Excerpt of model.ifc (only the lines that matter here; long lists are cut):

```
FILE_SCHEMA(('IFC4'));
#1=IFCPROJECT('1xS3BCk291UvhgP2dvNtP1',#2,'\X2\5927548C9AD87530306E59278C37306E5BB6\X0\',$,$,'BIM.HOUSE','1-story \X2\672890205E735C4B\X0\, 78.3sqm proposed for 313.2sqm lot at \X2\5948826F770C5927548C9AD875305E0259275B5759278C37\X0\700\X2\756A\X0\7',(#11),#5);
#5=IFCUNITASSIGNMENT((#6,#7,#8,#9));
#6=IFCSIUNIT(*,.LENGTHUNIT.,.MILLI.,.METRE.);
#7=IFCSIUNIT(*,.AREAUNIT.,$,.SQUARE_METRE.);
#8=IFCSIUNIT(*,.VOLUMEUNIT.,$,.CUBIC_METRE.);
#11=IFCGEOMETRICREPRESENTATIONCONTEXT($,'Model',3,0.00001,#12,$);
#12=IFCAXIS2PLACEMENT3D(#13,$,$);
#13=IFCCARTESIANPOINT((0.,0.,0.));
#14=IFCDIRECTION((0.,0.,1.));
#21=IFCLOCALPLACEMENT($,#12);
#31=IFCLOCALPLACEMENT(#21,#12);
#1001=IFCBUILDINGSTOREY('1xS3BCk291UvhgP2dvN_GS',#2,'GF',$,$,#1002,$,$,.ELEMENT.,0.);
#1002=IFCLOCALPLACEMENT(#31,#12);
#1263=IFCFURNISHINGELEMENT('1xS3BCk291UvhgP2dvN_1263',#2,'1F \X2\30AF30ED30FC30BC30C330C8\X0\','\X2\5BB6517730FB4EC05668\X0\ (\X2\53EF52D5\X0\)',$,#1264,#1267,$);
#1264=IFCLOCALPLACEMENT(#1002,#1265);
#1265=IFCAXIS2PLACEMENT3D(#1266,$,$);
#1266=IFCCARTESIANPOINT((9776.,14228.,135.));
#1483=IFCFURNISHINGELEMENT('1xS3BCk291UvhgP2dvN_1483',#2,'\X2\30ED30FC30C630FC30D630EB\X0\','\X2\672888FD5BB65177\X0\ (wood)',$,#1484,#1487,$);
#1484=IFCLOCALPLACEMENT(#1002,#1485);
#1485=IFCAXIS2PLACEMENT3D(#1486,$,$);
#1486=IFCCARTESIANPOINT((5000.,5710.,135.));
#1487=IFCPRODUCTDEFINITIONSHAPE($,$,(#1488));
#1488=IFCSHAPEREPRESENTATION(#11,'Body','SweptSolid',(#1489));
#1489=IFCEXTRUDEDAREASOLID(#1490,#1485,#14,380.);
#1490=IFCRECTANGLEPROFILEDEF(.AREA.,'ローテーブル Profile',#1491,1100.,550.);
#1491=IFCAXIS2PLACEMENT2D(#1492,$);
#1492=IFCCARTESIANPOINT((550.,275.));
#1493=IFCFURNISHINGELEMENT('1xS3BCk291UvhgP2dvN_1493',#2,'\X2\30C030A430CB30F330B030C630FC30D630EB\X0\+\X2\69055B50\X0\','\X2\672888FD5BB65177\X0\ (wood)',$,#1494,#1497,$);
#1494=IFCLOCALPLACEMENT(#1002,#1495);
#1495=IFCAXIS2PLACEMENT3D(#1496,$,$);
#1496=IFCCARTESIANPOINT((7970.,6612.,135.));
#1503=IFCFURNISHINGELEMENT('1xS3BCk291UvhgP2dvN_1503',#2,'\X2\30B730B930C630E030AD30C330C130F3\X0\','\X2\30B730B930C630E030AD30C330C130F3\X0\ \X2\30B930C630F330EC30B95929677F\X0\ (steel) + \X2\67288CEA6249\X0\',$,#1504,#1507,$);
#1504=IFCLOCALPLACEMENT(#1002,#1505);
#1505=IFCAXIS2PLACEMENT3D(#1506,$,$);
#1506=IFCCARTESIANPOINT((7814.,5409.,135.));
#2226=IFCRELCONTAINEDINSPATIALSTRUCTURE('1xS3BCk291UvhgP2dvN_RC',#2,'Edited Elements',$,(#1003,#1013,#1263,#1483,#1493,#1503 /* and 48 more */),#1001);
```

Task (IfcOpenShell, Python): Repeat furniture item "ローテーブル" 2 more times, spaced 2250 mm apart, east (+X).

```python
import numpy as np
import ifcopenshell
import ifcopenshell.api.geometry
import ifcopenshell.api.root
import ifcopenshell.util.element
import ifcopenshell.util.placement
import ifcopenshell.util.unit

model = ifcopenshell.open("model.ifc")
unit_scale = ifcopenshell.util.unit.calculate_unit_scale(model)


def reuse_history(source, copy):
    """copy_class also copies each property set's owner history, people and application; keep the originals."""
    for rel in copy.IsDefinedBy:
        if rel.is_a("IfcRelDefinesByProperties") and (history := rel.RelatingPropertyDefinition.OwnerHistory):
            rel.RelatingPropertyDefinition.OwnerHistory = source.OwnerHistory
            ifcopenshell.util.element.remove_deep2(model, history)


source = model.by_guid("1xS3BCk291UvhgP2dvN_1483")
base = ifcopenshell.util.placement.get_local_placement(source.ObjectPlacement)
step = np.array([1.0, 0.0, 0.0]) * 2.25 / unit_scale

for i in range(1, 3):
    copy = ifcopenshell.api.root.copy_class(model, product=source)
    copy.Representation = ifcopenshell.util.element.copy_deep(
        model, source.Representation, exclude=["IfcGeometricRepresentationContext", "IfcRepresentationMap"]
    )
    reuse_history(source, copy)
    matrix = base.copy()
    matrix[:3, 3] += i * step
    print("added at", matrix[:3, 3].round(3) + 0.0)
    ifcopenshell.api.geometry.edit_object_placement(model, product=copy, matrix=matrix, is_si=False)

model.write("model_updated.ifc")
```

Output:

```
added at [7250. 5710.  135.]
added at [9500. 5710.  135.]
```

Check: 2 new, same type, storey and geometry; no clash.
